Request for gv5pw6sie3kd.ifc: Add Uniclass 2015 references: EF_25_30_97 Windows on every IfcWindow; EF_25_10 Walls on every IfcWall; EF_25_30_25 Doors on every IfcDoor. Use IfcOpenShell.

First a look at what the model holds.

```python
import ifcopenshell

model = ifcopenshell.open("gv5pw6sie3kd.ifc")
print(model.schema)
print("classifications:", [c.Name for c in model.by_type("IfcClassification")])
for ifc_class in ("IfcDoor", "IfcRoof", "IfcStair", "IfcWall", "IfcWindow"):
    print(ifc_class, len(model.by_type(ifc_class)))
```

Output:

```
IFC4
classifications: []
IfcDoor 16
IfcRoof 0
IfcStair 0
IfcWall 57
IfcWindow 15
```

```python
import ifcopenshell
import ifcopenshell.api.classification

model = ifcopenshell.open("gv5pw6sie3kd.ifc")

system = ifcopenshell.api.classification.add_classification(model, classification="Uniclass 2015")

codes = {
    "IfcWindow": ("EF_25_30_97", "Windows"),
    "IfcWall": ("EF_25_10", "Walls"),
    "IfcDoor": ("EF_25_30_25", "Doors"),
}
for ifc_class, (code, name) in codes.items():
    products = model.by_type(ifc_class)
    ifcopenshell.api.classification.add_reference(
        model, products=products, classification=system, identification=code, name=name
    )
    print(code, len(products))

model.write("gv5pw6sie3kd_v2.ifc")
```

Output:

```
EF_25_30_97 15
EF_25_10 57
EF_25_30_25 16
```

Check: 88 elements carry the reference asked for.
